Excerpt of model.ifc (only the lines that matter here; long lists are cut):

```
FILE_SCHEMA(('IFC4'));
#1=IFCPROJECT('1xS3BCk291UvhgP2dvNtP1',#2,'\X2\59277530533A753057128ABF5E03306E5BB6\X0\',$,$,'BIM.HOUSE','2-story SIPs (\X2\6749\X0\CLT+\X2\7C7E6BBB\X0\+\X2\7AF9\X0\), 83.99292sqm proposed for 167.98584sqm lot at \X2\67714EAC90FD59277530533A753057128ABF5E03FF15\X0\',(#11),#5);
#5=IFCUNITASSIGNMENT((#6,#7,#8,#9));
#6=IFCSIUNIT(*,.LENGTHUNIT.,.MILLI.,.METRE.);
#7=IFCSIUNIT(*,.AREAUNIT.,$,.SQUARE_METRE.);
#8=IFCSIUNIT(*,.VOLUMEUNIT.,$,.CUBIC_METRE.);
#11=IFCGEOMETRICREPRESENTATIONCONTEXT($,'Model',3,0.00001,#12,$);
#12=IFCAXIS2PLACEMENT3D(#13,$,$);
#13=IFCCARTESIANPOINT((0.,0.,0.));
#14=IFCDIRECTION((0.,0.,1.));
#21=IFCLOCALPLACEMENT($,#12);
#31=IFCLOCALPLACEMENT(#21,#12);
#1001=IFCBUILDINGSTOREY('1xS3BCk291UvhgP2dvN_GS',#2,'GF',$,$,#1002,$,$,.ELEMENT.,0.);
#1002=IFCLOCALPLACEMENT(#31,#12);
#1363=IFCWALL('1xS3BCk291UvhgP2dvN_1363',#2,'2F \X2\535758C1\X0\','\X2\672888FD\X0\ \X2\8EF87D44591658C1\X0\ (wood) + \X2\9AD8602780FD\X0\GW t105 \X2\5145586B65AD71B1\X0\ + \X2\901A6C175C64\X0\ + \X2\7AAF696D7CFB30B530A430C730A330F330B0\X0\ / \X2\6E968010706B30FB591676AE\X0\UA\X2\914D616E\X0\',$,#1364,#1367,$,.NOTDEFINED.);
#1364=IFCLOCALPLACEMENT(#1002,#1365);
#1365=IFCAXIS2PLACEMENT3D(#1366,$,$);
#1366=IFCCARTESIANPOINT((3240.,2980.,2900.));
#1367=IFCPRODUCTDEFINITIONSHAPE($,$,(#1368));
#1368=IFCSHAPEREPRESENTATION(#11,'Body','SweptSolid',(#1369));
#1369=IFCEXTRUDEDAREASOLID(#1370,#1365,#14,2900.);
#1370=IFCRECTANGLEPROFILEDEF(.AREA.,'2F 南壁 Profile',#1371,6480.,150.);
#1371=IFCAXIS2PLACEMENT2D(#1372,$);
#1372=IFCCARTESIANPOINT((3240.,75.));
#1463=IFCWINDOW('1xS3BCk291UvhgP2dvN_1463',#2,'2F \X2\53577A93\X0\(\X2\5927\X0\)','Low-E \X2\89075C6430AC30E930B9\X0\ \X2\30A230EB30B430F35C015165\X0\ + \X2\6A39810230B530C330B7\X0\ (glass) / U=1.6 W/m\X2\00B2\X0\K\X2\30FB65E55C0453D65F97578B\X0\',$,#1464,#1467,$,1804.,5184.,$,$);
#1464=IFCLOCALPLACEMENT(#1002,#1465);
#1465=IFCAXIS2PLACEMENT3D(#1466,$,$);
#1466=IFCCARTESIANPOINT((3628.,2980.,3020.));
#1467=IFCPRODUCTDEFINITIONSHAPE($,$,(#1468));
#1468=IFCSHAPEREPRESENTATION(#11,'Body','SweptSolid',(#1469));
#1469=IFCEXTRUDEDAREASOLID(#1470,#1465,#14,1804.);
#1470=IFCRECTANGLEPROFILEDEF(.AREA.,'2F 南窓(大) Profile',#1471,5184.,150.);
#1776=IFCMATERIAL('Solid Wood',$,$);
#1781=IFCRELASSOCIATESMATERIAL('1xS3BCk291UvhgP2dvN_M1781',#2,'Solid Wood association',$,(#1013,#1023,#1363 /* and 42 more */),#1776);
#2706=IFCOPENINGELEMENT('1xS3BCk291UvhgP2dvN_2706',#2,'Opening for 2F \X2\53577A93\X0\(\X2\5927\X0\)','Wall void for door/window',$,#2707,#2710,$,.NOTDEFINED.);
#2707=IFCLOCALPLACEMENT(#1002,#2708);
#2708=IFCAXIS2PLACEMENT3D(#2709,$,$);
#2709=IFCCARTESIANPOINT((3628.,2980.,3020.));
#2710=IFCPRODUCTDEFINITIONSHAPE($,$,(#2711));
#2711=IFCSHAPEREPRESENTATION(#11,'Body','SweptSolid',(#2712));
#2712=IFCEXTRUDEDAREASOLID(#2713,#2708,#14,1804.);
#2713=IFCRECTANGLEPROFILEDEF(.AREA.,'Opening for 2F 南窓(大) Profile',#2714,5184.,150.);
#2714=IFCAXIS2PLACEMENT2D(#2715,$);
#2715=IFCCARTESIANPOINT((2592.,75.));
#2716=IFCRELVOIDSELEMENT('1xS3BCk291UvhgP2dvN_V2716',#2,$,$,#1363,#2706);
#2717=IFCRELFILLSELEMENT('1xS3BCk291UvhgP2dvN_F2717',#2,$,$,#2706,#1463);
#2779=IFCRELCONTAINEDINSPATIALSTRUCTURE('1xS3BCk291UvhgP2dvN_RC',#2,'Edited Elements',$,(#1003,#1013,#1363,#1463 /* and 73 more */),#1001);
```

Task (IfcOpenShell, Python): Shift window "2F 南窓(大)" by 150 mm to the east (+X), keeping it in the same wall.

```python
import ifcopenshell
import ifcopenshell.api.geometry
import ifcopenshell.util.placement
import ifcopenshell.util.unit

model = ifcopenshell.open("model.ifc")
unit_scale = ifcopenshell.util.unit.calculate_unit_scale(model)

window = model.by_id(1463)
opening = window.FillsVoids[0].RelatingOpeningElement
wall = opening.VoidsElements[0].RelatingBuildingElement

wall_matrix = ifcopenshell.util.placement.get_local_placement(wall.ObjectPlacement)
shift = wall_matrix[:3, 0] * 0.15 / unit_scale
before = ifcopenshell.util.placement.get_local_placement(window.ObjectPlacement)[:3, 3].copy()

# The window is not placed relative to its opening, so move both.
for product in (opening, window):
    matrix = ifcopenshell.util.placement.get_local_placement(product.ObjectPlacement)
    matrix[:3, 3] += shift
    ifcopenshell.api.geometry.edit_object_placement(model, product=product, matrix=matrix, is_si=False)

after = ifcopenshell.util.placement.get_local_placement(window.ObjectPlacement)[:3, 3]
print("window moved by", (after - before).round(3) + 0.0)

model.write("model_v2.ifc")
```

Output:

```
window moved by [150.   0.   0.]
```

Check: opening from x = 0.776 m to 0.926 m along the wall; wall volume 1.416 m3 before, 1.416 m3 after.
